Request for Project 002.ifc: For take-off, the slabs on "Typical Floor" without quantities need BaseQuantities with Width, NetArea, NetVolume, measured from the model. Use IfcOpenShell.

First a look at what the model holds.

```python
import ifcopenshell
import ifcopenshell.util.element
import ifcopenshell.util.unit

model = ifcopenshell.open("Project 002.ifc")
print(model.schema)
for unit_type in ("LENGTHUNIT", "AREAUNIT", "VOLUMEUNIT"):
    print(unit_type, ifcopenshell.util.unit.calculate_unit_scale(model, unit_type))
storey = next(s for s in model.by_type("IfcBuildingStorey") if s.Name == "Typical Floor")
slabs = [e for e in ifcopenshell.util.element.get_decomposition(storey) if e.is_a("IfcSlab")]
for e in sorted(slabs, key=lambda e: e.id()):
    print(e.id(), e.is_a(), e.Name, list(ifcopenshell.util.element.get_psets(e, qtos_only=True)), sep=" | ")
```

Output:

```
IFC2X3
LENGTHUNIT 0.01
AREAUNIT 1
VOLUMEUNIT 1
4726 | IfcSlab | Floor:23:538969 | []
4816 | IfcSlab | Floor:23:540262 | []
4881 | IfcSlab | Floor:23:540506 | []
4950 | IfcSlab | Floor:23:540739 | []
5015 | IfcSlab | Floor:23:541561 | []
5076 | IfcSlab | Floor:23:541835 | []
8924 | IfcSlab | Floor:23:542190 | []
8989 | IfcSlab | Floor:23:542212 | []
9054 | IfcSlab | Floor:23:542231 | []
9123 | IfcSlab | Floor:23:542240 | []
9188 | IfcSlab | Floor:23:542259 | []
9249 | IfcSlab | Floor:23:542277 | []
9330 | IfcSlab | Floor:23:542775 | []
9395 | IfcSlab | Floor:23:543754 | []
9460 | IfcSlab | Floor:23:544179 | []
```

```python
import ifcopenshell
import ifcopenshell.api.pset
import ifcopenshell.geom
import ifcopenshell.util.element
import ifcopenshell.util.shape
import ifcopenshell.util.unit

model = ifcopenshell.open("Project 002.ifc")
unit_scale = ifcopenshell.util.unit.calculate_unit_scale(model)
area_scale = ifcopenshell.util.unit.calculate_unit_scale(model, "AREAUNIT")
volume_scale = ifcopenshell.util.unit.calculate_unit_scale(model, "VOLUMEUNIT")
settings = ifcopenshell.geom.settings()

storey = next(s for s in model.by_type("IfcBuildingStorey") if s.Name == "Typical Floor")
slabs = [e for e in ifcopenshell.util.element.get_decomposition(storey) if e.is_a("IfcSlab")]

for e in sorted(slabs, key=lambda e: e.id()):
    if ifcopenshell.util.element.get_psets(e, qtos_only=True, should_inherit=False):
        continue
    # Geometry comes back in metres, in the element's own axes.
    shape = ifcopenshell.geom.create_shape(settings, e)
    values = {
        "Width": ifcopenshell.util.shape.get_z(shape.geometry) / unit_scale,
        "NetArea": ifcopenshell.util.shape.get_footprint_area(shape.geometry) / area_scale,
        "NetVolume": ifcopenshell.util.shape.get_volume(shape.geometry) / volume_scale,
    }
    qto = ifcopenshell.api.pset.add_qto(model, product=e, name="BaseQuantities")
    ifcopenshell.api.pset.edit_qto(model, qto=qto, properties=values)
    print(e.id(), {k: round(v, 3) for k, v in values.items()})

model.write("Project 002_edited.ifc")
```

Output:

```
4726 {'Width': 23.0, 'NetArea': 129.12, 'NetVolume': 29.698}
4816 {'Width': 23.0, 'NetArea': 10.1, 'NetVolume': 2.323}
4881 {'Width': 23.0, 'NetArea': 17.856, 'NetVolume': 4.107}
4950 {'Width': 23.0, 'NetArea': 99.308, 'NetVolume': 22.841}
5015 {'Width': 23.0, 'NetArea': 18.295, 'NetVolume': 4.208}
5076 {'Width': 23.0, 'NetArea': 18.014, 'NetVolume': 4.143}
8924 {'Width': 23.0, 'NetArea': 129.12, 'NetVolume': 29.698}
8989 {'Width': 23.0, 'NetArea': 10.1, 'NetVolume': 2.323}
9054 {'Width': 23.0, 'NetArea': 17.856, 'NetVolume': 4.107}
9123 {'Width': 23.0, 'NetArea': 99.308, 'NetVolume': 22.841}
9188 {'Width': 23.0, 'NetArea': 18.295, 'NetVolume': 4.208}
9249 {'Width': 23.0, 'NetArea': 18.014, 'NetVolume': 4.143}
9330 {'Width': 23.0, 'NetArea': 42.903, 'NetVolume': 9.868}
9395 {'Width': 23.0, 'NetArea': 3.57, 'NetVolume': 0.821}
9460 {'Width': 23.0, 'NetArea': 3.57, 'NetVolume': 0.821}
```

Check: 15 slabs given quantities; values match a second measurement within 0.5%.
